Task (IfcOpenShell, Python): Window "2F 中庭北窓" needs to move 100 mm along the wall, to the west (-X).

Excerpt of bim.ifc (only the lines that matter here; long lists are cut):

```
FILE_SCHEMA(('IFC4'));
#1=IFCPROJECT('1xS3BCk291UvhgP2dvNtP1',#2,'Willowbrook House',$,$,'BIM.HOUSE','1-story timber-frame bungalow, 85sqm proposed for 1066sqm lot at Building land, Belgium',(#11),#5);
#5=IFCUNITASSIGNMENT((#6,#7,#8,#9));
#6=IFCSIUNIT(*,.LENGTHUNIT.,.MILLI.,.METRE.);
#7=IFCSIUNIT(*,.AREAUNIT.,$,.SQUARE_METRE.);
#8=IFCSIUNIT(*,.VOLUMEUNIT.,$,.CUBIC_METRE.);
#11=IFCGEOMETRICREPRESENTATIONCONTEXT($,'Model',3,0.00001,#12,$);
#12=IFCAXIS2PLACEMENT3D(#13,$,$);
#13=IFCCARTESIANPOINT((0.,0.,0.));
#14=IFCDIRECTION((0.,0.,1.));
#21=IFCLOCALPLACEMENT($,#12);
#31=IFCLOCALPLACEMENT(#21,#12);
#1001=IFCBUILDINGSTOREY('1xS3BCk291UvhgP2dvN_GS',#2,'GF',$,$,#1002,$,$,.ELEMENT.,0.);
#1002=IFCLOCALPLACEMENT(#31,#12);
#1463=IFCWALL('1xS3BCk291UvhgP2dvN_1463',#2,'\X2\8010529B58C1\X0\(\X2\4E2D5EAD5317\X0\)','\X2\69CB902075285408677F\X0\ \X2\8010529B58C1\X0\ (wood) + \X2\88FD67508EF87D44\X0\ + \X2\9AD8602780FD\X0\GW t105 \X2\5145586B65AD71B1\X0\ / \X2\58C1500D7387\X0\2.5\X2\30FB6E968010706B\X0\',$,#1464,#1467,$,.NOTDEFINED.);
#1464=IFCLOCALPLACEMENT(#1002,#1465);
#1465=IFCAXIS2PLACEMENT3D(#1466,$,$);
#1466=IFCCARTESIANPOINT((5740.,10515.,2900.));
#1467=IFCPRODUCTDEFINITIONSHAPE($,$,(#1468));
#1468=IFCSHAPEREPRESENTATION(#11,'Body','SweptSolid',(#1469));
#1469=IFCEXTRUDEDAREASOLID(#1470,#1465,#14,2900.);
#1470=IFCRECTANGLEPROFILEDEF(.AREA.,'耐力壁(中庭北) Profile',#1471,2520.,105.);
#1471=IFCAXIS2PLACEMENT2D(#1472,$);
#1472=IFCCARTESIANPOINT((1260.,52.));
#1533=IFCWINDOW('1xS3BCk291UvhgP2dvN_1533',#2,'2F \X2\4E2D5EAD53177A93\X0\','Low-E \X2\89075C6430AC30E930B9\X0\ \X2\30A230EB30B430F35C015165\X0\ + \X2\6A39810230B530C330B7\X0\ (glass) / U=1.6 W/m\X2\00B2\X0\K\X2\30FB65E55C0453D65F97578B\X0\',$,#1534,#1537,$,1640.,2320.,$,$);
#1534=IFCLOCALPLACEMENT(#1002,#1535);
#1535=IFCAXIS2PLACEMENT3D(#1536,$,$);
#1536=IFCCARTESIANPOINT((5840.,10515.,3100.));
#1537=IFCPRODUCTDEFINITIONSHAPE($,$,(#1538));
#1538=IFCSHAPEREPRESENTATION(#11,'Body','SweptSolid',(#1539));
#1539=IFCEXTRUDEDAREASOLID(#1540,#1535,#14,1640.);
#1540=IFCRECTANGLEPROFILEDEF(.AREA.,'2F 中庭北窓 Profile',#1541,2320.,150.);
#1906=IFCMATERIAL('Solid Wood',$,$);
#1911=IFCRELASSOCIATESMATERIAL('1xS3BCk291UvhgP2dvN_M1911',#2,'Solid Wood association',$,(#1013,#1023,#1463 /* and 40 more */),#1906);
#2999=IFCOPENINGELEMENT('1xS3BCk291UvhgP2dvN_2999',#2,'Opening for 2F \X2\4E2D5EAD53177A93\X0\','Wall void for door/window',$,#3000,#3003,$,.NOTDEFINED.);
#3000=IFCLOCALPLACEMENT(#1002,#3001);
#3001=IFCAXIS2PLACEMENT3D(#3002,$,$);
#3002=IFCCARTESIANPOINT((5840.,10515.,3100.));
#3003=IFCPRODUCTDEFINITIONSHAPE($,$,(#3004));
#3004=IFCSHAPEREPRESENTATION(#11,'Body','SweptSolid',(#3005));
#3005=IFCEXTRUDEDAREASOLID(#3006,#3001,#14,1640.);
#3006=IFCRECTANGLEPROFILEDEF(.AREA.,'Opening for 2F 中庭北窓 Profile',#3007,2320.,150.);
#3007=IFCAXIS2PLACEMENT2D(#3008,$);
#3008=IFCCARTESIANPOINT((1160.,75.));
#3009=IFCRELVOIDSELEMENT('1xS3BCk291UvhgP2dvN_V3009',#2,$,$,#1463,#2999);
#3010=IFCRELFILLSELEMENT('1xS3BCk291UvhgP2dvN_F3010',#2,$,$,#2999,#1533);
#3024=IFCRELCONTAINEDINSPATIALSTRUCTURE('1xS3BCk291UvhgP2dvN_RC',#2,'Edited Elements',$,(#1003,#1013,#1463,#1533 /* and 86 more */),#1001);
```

```python
import ifcopenshell
import ifcopenshell.api.geometry
import ifcopenshell.util.placement
import ifcopenshell.util.unit

model = ifcopenshell.open("bim.ifc")
unit_scale = ifcopenshell.util.unit.calculate_unit_scale(model)

window = model.by_id(1533)
opening = window.FillsVoids[0].RelatingOpeningElement
wall = opening.VoidsElements[0].RelatingBuildingElement

wall_matrix = ifcopenshell.util.placement.get_local_placement(wall.ObjectPlacement)
shift = wall_matrix[:3, 0] * -0.1 / unit_scale
before = ifcopenshell.util.placement.get_local_placement(window.ObjectPlacement)[:3, 3].copy()

# The window is not placed relative to its opening, so move both.
for product in (opening, window):
    matrix = ifcopenshell.util.placement.get_local_placement(product.ObjectPlacement)
    matrix[:3, 3] += shift
    ifcopenshell.api.geometry.edit_object_placement(model, product=product, matrix=matrix, is_si=False)

after = ifcopenshell.util.placement.get_local_placement(window.ObjectPlacement)[:3, 3]
print("window moved by", (after - before).round(3) + 0.0)

model.write("bim_updated.ifc")
```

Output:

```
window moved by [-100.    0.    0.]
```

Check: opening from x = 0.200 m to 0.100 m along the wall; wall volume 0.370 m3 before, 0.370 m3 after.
